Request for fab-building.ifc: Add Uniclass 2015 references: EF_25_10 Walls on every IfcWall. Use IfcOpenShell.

First a look at what the model holds.

```python
import ifcopenshell

model = ifcopenshell.open("fab-building.ifc")
print(model.schema)
print("classifications:", [c.Name for c in model.by_type("IfcClassification")])
for ifc_class in ("IfcDoor", "IfcRoof", "IfcStair", "IfcWall", "IfcWindow"):
    print(ifc_class, len(model.by_type(ifc_class)))
```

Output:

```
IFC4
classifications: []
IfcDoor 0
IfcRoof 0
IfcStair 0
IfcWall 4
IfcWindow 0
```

```python
import ifcopenshell
import ifcopenshell.api.classification

model = ifcopenshell.open("fab-building.ifc")

system = ifcopenshell.api.classification.add_classification(model, classification="Uniclass 2015")

codes = {
    "IfcWall": ("EF_25_10", "Walls"),
}
for ifc_class, (code, name) in codes.items():
    products = model.by_type(ifc_class)
    ifcopenshell.api.classification.add_reference(
        model, products=products, classification=system, identification=code, name=name
    )
    print(code, len(products))

model.write("fab-building-out.ifc")
```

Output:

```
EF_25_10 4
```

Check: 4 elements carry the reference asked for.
